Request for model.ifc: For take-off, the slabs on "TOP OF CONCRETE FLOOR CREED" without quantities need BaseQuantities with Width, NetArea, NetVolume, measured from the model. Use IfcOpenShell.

First a look at what the model holds.

```python
import ifcopenshell
import ifcopenshell.util.element
import ifcopenshell.util.unit

model = ifcopenshell.open("model.ifc")
print(model.schema)
for unit_type in ("LENGTHUNIT", "AREAUNIT", "VOLUMEUNIT"):
    print(unit_type, ifcopenshell.util.unit.calculate_unit_scale(model, unit_type))
storey = next(s for s in model.by_type("IfcBuildingStorey") if s.Name == "TOP OF CONCRETE FLOOR CREED")
slabs = [e for e in ifcopenshell.util.element.get_decomposition(storey) if e.is_a("IfcSlab")]
for e in sorted(slabs, key=lambda e: e.id()):
    print(e.id(), e.is_a(), e.Name, list(ifcopenshell.util.element.get_psets(e, qtos_only=True)), sep=" | ")
```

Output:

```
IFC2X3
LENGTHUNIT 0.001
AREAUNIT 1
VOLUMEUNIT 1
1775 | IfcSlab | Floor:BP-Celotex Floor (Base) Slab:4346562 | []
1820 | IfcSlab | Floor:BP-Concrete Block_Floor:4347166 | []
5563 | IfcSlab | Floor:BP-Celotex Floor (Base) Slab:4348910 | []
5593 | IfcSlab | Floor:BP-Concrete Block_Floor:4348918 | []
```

```python
import ifcopenshell
import ifcopenshell.api.pset
import ifcopenshell.geom
import ifcopenshell.util.element
import ifcopenshell.util.shape
import ifcopenshell.util.unit

model = ifcopenshell.open("model.ifc")
unit_scale = ifcopenshell.util.unit.calculate_unit_scale(model)
area_scale = ifcopenshell.util.unit.calculate_unit_scale(model, "AREAUNIT")
volume_scale = ifcopenshell.util.unit.calculate_unit_scale(model, "VOLUMEUNIT")
settings = ifcopenshell.geom.settings()

storey = next(s for s in model.by_type("IfcBuildingStorey") if s.Name == "TOP OF CONCRETE FLOOR CREED")
slabs = [e for e in ifcopenshell.util.element.get_decomposition(storey) if e.is_a("IfcSlab")]

for e in sorted(slabs, key=lambda e: e.id()):
    if ifcopenshell.util.element.get_psets(e, qtos_only=True, should_inherit=False):
        continue
    # Geometry comes back in metres, in the element's own axes.
    shape = ifcopenshell.geom.create_shape(settings, e)
    values = {
        "Width": ifcopenshell.util.shape.get_z(shape.geometry) / unit_scale,
        "NetArea": ifcopenshell.util.shape.get_footprint_area(shape.geometry) / area_scale,
        "NetVolume": ifcopenshell.util.shape.get_volume(shape.geometry) / volume_scale,
    }
    qto = ifcopenshell.api.pset.add_qto(model, product=e, name="BaseQuantities")
    ifcopenshell.api.pset.edit_qto(model, qto=qto, properties=values)
    print(e.id(), {k: round(v, 3) for k, v in values.items()})

model.write("model_rev.ifc")
```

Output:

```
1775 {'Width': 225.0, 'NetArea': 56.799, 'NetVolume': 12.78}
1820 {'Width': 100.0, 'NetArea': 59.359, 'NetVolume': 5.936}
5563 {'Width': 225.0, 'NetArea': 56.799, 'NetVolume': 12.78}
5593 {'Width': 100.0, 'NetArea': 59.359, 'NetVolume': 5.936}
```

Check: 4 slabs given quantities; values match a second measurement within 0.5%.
